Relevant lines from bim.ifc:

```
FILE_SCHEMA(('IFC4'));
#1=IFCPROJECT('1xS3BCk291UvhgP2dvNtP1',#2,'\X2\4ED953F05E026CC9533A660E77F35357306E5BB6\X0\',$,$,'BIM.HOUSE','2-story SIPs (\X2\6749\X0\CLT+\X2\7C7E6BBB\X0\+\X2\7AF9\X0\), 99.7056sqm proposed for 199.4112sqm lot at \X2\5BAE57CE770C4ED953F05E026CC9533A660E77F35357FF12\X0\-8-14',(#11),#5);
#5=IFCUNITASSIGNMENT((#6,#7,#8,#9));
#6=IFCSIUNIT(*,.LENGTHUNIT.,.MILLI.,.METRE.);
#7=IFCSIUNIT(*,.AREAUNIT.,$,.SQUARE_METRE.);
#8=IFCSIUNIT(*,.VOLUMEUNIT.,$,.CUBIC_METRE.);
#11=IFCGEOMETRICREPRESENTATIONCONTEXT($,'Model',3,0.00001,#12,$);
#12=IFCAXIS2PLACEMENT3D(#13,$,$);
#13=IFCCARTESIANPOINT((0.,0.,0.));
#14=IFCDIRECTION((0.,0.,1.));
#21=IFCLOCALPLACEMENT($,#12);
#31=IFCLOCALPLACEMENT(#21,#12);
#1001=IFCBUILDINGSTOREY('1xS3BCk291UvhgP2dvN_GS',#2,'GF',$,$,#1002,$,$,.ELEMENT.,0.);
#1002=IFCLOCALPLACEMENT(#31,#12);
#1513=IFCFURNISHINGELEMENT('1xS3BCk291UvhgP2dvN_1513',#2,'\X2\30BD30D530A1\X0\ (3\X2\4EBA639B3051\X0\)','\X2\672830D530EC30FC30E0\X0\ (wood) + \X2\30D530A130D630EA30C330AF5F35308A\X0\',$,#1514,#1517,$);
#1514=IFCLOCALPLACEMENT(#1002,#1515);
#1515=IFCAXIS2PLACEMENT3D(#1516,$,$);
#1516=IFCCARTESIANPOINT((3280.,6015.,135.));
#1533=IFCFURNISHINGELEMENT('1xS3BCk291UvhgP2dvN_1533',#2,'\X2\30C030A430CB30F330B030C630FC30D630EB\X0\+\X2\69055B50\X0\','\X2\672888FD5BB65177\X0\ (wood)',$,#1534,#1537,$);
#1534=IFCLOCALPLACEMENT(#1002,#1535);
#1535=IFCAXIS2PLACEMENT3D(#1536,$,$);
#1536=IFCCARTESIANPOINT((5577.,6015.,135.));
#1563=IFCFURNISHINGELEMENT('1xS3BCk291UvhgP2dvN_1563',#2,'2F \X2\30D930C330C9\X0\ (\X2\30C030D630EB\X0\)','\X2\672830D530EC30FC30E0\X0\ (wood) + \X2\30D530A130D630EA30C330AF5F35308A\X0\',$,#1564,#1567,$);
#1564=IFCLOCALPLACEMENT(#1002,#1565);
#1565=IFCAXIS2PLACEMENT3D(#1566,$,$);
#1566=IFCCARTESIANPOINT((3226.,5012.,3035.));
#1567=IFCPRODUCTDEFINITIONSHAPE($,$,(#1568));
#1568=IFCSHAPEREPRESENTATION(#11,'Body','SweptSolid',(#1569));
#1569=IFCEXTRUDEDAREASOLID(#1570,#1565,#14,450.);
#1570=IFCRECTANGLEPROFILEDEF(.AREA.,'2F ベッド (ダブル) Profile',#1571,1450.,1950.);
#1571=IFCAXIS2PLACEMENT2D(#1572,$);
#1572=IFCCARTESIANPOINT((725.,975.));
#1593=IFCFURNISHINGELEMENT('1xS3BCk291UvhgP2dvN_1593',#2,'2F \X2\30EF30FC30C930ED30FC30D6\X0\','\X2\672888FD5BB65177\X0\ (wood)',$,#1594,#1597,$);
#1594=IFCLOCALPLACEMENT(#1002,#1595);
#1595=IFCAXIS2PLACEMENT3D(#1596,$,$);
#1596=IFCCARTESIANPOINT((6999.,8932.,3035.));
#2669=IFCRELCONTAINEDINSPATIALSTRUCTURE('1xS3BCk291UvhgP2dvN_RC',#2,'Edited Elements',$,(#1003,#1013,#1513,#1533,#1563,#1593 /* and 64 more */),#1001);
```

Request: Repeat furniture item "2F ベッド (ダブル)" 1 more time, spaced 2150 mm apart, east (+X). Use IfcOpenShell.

```python
import numpy as np
import ifcopenshell
import ifcopenshell.api.geometry
import ifcopenshell.api.root
import ifcopenshell.util.element
import ifcopenshell.util.placement
import ifcopenshell.util.unit

model = ifcopenshell.open("bim.ifc")
unit_scale = ifcopenshell.util.unit.calculate_unit_scale(model)


def reuse_history(source, copy):
    """copy_class also copies each property set's owner history, people and application; keep the originals."""
    for rel in copy.IsDefinedBy:
        if rel.is_a("IfcRelDefinesByProperties") and (history := rel.RelatingPropertyDefinition.OwnerHistory):
            rel.RelatingPropertyDefinition.OwnerHistory = source.OwnerHistory
            ifcopenshell.util.element.remove_deep2(model, history)


source = model.by_id(1563)
base = ifcopenshell.util.placement.get_local_placement(source.ObjectPlacement)
step = np.array([1.0, 0.0, 0.0]) * 2.15 / unit_scale

for i in range(1, 2):
    copy = ifcopenshell.api.root.copy_class(model, product=source)
    copy.Representation = ifcopenshell.util.element.copy_deep(
        model, source.Representation, exclude=["IfcGeometricRepresentationContext", "IfcRepresentationMap"]
    )
    reuse_history(source, copy)
    matrix = base.copy()
    matrix[:3, 3] += i * step
    print("added at", matrix[:3, 3].round(3) + 0.0)
    ifcopenshell.api.geometry.edit_object_placement(model, product=copy, matrix=matrix, is_si=False)

model.write("bim_updated.ifc")
```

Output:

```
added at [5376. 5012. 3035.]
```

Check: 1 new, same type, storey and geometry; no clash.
